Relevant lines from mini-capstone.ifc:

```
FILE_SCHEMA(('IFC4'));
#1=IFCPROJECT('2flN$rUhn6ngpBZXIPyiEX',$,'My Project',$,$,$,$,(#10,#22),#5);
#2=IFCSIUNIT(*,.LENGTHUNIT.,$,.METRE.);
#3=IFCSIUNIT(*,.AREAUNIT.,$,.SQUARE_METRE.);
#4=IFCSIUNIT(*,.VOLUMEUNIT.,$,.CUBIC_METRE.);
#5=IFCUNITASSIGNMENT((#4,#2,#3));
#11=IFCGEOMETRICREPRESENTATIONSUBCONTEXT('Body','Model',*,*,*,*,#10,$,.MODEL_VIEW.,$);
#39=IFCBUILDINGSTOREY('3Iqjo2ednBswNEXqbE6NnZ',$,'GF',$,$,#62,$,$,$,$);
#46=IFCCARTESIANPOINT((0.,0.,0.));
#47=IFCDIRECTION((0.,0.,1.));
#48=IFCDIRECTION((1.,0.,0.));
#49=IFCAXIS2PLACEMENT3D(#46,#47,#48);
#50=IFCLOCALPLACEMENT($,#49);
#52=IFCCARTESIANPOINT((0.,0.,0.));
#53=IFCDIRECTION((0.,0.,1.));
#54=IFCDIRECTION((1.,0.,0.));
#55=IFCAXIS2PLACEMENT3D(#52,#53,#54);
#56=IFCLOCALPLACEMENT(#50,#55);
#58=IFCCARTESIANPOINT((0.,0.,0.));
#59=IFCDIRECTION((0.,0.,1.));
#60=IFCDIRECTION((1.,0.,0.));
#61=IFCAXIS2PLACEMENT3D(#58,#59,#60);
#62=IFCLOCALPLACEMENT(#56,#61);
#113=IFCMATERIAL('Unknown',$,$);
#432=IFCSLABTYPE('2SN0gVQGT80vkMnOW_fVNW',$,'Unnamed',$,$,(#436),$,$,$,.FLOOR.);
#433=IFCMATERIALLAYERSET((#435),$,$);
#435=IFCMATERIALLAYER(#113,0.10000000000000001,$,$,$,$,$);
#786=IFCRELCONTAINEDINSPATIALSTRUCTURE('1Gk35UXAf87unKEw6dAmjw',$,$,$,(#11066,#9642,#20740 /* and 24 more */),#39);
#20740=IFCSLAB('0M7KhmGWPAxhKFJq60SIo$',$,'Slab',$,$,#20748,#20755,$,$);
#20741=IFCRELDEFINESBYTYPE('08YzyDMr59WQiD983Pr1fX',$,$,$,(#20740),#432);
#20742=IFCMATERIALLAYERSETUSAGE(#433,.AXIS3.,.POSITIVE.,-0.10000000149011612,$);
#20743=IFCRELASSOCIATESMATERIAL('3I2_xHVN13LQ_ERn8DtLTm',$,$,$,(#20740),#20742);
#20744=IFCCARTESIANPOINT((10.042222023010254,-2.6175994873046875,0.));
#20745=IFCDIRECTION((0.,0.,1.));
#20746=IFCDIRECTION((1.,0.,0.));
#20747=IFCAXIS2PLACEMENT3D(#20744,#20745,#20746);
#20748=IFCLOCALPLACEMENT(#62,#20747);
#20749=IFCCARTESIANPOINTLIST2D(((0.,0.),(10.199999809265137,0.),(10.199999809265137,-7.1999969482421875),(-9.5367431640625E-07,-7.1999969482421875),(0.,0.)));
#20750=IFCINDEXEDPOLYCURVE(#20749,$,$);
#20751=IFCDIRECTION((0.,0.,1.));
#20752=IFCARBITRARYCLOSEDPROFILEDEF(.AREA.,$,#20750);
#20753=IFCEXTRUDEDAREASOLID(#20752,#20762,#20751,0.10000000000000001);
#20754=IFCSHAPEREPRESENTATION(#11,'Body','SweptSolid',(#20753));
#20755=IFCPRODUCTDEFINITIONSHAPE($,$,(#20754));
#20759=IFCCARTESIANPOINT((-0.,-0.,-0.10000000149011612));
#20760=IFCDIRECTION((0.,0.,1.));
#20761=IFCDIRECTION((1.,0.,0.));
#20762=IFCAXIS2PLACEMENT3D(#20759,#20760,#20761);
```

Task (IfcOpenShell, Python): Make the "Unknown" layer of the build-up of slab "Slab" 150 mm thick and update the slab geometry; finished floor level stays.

```python
import ifcopenshell
import ifcopenshell.util.element
import ifcopenshell.util.representation
import ifcopenshell.util.unit

model = ifcopenshell.open("mini-capstone.ifc")
unit_scale = ifcopenshell.util.unit.calculate_unit_scale(model)

layer_set = model.by_id(433)
layer = next(l for l in layer_set.MaterialLayers if l.Material and l.Material.Name == "Unknown")
change = 0.15 / unit_scale - layer.LayerThickness
layer.LayerThickness += change

# Geometry does not follow the layer set by itself.
slabs = [e for e in ifcopenshell.util.element.get_elements_by_material(model, layer_set) if e.is_a("IfcSlab")]
for slab in sorted(slabs, key=lambda e: e.id()):
    body = ifcopenshell.util.representation.get_representation(slab, "Model", "Body")
    solid = body.Items[0]
    old_depth = solid.Depth
    solid.Depth += change
    # Extruded upwards: lower the start of the extrusion so the top stays.
    x, y, z = solid.Position.Location.Coordinates
    solid.Position.Location = model.createIfcCartesianPoint((x, y, z - change))
    print(slab.id(), f"{old_depth:g} -> {solid.Depth:g}")

# The layers are counted up from the underside, which has moved.
for usage in {ifcopenshell.util.element.get_material(slab) for slab in slabs}:
    usage.OffsetFromReferenceLine -= change

model.write("mini-capstone_updated.ifc")
```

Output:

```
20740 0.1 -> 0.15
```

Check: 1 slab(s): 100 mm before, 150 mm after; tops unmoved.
